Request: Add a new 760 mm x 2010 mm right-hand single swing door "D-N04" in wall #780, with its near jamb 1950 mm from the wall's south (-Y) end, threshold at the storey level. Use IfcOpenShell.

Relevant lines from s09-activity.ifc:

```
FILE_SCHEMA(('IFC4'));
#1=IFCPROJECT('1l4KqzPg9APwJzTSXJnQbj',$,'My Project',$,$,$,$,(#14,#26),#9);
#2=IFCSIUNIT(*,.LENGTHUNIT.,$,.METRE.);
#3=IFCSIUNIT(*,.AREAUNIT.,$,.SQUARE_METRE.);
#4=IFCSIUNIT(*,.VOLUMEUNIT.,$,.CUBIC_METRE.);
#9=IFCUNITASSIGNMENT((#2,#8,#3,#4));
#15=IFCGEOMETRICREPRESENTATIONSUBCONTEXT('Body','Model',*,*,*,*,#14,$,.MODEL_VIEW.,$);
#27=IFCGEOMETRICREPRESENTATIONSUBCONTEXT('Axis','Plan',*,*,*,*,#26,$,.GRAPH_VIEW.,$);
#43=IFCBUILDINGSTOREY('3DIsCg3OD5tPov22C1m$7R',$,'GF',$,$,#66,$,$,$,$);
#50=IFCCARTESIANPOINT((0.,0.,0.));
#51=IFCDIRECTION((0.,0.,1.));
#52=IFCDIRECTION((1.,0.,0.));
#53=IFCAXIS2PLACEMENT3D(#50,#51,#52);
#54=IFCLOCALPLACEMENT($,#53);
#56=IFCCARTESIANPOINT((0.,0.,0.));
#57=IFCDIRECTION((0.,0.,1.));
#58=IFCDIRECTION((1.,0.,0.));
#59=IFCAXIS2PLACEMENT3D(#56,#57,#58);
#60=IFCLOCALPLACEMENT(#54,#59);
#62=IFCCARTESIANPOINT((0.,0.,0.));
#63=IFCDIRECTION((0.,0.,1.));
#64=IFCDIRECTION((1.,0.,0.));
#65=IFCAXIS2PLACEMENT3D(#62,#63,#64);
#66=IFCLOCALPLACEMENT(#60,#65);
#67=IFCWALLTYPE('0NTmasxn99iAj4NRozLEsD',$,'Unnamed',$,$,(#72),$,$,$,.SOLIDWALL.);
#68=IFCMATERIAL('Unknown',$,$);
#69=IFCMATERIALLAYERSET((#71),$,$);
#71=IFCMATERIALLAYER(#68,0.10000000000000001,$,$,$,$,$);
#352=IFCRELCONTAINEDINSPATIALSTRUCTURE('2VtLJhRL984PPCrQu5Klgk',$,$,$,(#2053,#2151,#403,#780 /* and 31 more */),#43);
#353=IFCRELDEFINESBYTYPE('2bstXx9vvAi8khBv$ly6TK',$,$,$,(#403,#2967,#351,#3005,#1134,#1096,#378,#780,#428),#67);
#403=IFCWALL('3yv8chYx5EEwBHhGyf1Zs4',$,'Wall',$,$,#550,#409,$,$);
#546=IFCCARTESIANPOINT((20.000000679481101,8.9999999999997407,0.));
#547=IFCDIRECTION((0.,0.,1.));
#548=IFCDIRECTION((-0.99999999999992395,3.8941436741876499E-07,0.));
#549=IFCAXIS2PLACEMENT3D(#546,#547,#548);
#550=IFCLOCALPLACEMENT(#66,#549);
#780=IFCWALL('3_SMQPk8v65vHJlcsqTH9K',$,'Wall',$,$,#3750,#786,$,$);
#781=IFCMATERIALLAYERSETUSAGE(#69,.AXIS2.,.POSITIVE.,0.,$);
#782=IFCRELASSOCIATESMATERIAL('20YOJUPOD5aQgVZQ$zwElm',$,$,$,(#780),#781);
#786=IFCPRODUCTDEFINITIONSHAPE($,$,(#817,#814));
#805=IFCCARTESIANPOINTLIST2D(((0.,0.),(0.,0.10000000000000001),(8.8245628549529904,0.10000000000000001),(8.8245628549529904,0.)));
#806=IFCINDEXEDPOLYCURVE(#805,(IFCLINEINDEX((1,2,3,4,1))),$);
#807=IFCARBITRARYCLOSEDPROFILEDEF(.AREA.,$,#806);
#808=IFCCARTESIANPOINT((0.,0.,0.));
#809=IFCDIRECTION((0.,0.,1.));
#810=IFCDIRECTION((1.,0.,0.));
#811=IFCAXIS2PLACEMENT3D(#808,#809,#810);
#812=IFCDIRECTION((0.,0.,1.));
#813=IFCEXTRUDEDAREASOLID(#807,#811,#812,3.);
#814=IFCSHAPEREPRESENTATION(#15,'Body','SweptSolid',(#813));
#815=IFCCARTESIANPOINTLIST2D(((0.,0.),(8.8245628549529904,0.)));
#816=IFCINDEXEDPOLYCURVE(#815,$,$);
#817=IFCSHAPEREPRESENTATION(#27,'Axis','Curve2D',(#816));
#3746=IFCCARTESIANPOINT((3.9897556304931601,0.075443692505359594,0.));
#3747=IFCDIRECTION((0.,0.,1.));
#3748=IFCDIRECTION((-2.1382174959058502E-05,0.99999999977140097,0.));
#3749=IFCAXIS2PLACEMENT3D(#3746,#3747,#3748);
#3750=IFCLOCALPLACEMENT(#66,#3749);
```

```python
import numpy as np
import ifcopenshell
import ifcopenshell.api.feature
import ifcopenshell.api.geometry
import ifcopenshell.api.root
import ifcopenshell.api.spatial
import ifcopenshell.geom
import ifcopenshell.util.element
import ifcopenshell.util.placement
import ifcopenshell.util.representation
import ifcopenshell.util.shape
import ifcopenshell.util.unit

model = ifcopenshell.open("s09-activity.ifc")
unit_scale = ifcopenshell.util.unit.calculate_unit_scale(model)
settings = ifcopenshell.geom.settings()


def volume(element):
    """Net volume in cubic metres, openings subtracted."""
    shape = ifcopenshell.geom.create_shape(settings, element)
    return ifcopenshell.util.shape.get_volume(shape.geometry)


wall = model.by_id(780)
storey = ifcopenshell.util.element.get_container(wall, ifc_class="IfcBuildingStorey")
context = ifcopenshell.util.representation.get_context(model, "Model", "Body", "MODEL_VIEW")
before = volume(wall)

width, height, from_end, sill = 0.76, 2.01, 1.95, 0.0  # metres

# The wall runs along its own X axis, and the end named is its -X end.
wall_shape = ifcopenshell.geom.create_shape(settings, wall)
x, y, z = ifcopenshell.util.shape.get_vertices(wall_shape.geometry).T
start = x.min() + from_end
face, thickness = float(y.min()), float(y.max() - y.min())
wall_matrix = ifcopenshell.util.placement.get_local_placement(wall.ObjectPlacement)
level = ifcopenshell.util.placement.get_local_placement(storey.ObjectPlacement)[2, 3]


def in_wall(x, y):
    """Placement at x, y metres in the wall's axes, at sill height."""
    matrix = wall_matrix.copy()
    matrix[:, 3] = wall_matrix @ np.array([x / unit_scale, y / unit_scale, 0.0, 1.0])
    matrix[2, 3] = level + sill / unit_scale
    return matrix


# Opening: a box that overshoots both wall faces by 50 mm.
opening = ifcopenshell.api.root.create_entity(model, ifc_class="IfcOpeningElement", predefined_type="OPENING")
box = ifcopenshell.api.geometry.add_wall_representation(
    model, context=context, length=width, height=height, thickness=thickness + 0.1
)
ifcopenshell.api.geometry.assign_representation(model, product=opening, representation=box)
ifcopenshell.api.geometry.edit_object_placement(model, product=opening, matrix=in_wall(start, face - 0.05), is_si=False)
ifcopenshell.api.feature.add_feature(model, feature=opening, element=wall)

door = ifcopenshell.api.root.create_entity(model, ifc_class="IfcDoor", name="D-N04", predefined_type="DOOR")
door.OverallWidth, door.OverallHeight = width / unit_scale, height / unit_scale
door.OperationType = "SINGLE_SWING_RIGHT"
body = ifcopenshell.api.geometry.add_door_representation(
    model,
    context=context,
    overall_width=door.OverallWidth,
    overall_height=door.OverallHeight,
    operation_type="SINGLE_SWING_RIGHT",
    lining_properties={"LiningDepth": thickness / unit_scale, "ThresholdDepth": thickness / unit_scale},
)
ifcopenshell.api.geometry.assign_representation(model, product=door, representation=body)
ifcopenshell.api.spatial.assign_container(model, products=[door], relating_structure=storey)
ifcopenshell.api.feature.add_filling(model, opening=opening, element=door)

# The lining spans the wall, so the door starts at the wall face.
ifcopenshell.api.geometry.edit_object_placement(model, product=door, matrix=in_wall(start, face), is_si=False)

after = volume(wall)

print(f"wall volume {before:.3f} -> {after:.3f} m3")

model.write("s09-activity_updated.ifc")
```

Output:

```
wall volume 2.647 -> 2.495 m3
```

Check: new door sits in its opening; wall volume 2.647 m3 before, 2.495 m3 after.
